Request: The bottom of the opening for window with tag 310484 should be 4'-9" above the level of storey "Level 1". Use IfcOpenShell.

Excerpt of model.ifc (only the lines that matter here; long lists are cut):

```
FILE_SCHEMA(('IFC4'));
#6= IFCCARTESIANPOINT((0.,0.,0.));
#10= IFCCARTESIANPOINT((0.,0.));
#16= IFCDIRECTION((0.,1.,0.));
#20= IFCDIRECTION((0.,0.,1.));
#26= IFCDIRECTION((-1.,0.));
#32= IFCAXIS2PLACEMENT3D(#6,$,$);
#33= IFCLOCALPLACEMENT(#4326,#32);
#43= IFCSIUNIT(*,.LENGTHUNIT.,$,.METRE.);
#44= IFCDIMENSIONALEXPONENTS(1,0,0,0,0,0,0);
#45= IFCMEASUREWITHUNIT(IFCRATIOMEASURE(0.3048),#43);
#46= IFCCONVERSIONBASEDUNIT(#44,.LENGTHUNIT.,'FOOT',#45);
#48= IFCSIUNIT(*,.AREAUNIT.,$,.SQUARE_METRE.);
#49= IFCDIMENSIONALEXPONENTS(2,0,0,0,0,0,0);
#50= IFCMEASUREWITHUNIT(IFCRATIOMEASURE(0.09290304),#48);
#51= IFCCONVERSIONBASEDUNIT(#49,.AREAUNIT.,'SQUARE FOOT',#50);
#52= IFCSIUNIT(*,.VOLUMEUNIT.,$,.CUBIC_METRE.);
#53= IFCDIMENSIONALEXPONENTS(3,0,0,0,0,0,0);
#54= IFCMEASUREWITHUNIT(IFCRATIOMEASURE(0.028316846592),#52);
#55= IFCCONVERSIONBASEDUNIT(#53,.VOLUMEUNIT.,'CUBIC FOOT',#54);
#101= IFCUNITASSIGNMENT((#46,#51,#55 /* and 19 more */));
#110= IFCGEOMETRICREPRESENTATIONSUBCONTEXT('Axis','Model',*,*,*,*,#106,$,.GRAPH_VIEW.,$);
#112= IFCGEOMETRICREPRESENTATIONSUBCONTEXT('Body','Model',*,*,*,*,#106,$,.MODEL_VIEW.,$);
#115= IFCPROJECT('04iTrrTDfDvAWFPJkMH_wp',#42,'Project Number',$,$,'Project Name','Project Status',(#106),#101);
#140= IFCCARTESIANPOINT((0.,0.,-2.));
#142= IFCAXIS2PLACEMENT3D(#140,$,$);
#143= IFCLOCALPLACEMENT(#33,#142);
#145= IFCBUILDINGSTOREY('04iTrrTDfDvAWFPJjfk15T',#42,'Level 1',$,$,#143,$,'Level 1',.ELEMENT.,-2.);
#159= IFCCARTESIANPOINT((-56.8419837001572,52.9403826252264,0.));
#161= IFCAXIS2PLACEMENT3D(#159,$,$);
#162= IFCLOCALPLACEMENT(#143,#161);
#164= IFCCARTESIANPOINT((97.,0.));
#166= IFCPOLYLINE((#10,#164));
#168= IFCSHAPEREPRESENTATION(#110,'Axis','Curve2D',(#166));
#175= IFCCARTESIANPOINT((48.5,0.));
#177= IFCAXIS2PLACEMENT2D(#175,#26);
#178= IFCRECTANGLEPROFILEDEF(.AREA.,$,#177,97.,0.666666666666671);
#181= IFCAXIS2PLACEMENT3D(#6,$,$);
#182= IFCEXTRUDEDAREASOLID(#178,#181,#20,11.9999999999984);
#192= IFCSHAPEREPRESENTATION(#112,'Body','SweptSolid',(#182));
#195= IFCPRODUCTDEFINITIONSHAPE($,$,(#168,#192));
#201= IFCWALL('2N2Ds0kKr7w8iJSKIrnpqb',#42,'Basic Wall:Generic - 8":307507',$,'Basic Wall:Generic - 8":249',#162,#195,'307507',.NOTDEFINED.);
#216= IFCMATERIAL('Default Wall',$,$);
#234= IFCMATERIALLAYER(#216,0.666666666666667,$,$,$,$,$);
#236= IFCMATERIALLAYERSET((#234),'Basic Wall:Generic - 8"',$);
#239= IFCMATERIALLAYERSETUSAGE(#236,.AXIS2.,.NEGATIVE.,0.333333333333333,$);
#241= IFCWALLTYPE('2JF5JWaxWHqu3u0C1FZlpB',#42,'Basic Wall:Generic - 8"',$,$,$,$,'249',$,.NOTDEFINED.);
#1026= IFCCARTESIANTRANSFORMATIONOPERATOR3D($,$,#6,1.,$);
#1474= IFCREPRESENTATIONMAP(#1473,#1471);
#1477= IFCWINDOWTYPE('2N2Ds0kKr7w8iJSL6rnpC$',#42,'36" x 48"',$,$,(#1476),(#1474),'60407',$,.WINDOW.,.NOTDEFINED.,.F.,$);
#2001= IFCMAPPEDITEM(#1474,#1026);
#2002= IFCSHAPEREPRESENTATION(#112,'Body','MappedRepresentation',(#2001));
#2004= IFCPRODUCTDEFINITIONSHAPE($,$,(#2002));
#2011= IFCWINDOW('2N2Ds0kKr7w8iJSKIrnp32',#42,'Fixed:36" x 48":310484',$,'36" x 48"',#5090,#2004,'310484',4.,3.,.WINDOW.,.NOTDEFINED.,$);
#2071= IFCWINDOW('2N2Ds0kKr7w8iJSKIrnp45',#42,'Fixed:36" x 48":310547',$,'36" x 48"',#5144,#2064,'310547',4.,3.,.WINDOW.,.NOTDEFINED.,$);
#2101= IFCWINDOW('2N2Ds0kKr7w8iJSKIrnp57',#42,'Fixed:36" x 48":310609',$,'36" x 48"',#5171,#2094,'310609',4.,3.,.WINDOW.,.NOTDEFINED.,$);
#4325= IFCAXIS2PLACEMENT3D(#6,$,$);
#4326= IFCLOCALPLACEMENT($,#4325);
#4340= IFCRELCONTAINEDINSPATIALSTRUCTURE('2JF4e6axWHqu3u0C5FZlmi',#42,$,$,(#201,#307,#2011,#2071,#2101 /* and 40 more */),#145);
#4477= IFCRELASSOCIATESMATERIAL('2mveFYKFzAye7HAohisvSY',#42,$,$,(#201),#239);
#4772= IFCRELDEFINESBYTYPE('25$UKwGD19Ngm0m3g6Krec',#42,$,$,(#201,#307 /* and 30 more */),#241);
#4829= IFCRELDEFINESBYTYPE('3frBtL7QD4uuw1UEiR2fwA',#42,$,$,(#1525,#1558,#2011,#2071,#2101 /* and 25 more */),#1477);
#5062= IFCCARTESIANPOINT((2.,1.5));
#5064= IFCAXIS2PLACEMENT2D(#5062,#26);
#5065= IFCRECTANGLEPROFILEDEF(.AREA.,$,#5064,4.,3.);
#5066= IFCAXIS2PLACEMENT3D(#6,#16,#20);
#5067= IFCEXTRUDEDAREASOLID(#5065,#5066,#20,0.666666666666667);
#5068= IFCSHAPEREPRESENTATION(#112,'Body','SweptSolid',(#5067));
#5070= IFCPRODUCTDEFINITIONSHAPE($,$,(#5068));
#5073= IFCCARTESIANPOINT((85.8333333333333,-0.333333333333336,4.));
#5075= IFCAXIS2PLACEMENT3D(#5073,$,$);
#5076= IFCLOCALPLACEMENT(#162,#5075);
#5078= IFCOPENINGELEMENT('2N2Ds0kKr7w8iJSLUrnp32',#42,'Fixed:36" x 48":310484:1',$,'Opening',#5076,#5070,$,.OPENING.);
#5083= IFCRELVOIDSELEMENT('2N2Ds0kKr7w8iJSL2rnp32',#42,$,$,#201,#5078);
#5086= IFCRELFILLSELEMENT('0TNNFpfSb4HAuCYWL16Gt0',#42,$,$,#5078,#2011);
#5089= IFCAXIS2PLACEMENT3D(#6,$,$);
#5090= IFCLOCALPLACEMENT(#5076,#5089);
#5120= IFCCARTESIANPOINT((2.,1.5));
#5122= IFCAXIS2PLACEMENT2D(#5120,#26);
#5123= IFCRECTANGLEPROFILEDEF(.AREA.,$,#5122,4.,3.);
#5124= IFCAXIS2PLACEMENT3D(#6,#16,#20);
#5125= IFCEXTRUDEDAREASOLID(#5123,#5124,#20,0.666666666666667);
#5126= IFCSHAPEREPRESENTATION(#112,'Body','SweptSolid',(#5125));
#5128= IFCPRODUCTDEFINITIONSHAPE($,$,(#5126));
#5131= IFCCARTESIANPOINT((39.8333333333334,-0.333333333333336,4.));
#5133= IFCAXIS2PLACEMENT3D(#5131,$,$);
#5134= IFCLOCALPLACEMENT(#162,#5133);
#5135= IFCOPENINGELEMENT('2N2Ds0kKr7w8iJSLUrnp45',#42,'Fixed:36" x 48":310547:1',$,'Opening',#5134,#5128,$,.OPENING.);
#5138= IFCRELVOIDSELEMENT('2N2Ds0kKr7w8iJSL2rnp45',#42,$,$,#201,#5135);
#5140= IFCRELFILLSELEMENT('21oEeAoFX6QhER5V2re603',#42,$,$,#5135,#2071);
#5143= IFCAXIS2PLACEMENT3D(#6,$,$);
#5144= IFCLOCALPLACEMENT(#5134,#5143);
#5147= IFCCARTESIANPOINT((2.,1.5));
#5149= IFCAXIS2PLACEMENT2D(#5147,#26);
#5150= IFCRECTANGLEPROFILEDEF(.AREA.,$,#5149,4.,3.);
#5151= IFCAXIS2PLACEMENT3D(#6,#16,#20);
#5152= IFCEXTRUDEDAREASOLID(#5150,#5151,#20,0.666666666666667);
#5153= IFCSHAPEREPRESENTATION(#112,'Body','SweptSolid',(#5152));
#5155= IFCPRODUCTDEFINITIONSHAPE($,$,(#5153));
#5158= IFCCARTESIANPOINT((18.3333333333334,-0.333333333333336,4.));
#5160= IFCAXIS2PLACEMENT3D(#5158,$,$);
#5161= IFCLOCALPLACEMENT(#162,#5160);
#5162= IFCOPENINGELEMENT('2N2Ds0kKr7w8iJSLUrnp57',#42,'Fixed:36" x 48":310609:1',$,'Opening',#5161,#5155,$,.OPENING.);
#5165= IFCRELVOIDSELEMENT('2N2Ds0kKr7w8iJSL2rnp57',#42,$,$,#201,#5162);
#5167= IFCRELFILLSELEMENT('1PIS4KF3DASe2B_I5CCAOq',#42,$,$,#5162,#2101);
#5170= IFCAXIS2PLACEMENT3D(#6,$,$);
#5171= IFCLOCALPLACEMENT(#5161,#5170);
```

```python
import numpy as np
import ifcopenshell
import ifcopenshell.api.geometry
import ifcopenshell.geom
import ifcopenshell.util.element
import ifcopenshell.util.placement
import ifcopenshell.util.shape
import ifcopenshell.util.unit

model = ifcopenshell.open("model.ifc")
unit_scale = ifcopenshell.util.unit.calculate_unit_scale(model)

window = model.by_id(2011)
opening = window.FillsVoids[0].RelatingOpeningElement
storey = ifcopenshell.util.element.get_container(window, ifc_class="IfcBuildingStorey")
level = ifcopenshell.util.placement.get_local_placement(storey.ObjectPlacement)[2, 3]

# The opening's origin need not be at the sill, so measure its lowest point.
shape = ifcopenshell.geom.create_shape(ifcopenshell.geom.settings(), opening)
bottom = ifcopenshell.util.shape.get_shape_bottom_elevation(shape, shape.geometry) / unit_scale
dz = level + 57 * 0.0254 / unit_scale - bottom

shift = np.array([0.0, 0.0, dz])
# The window is placed relative to its opening, so it follows when the opening moves.
matrix = ifcopenshell.util.placement.get_local_placement(opening.ObjectPlacement)
matrix[:3, 3] += shift
ifcopenshell.api.geometry.edit_object_placement(
    model, product=opening, matrix=matrix, is_si=False, should_transform_children=True
)

print(f"moved by {dz * unit_scale:+.3f} m")

model.write("model_edited.ifc")
```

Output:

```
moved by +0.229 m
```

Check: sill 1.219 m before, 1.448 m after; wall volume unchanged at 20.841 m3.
